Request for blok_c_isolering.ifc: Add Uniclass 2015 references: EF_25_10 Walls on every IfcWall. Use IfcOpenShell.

First a look at what the model holds.

```python
import ifcopenshell

model = ifcopenshell.open("blok_c_isolering.ifc")
print(model.schema)
print("classifications:", [c.Name for c in model.by_type("IfcClassification")])
for ifc_class in ("IfcDoor", "IfcRoof", "IfcStair", "IfcWall", "IfcWindow"):
    print(ifc_class, len(model.by_type(ifc_class)))
```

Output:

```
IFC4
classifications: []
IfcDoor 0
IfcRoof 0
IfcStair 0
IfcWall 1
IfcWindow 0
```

```python
import ifcopenshell
import ifcopenshell.api.classification

model = ifcopenshell.open("blok_c_isolering.ifc")

system = ifcopenshell.api.classification.add_classification(model, classification="Uniclass 2015")

codes = {
    "IfcWall": ("EF_25_10", "Walls"),
}
for ifc_class, (code, name) in codes.items():
    products = model.by_type(ifc_class)
    ifcopenshell.api.classification.add_reference(
        model, products=products, classification=system, identification=code, name=name
    )
    print(code, len(products))

model.write("blok_c_isolering_v2.ifc")
```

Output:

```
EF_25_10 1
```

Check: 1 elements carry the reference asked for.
